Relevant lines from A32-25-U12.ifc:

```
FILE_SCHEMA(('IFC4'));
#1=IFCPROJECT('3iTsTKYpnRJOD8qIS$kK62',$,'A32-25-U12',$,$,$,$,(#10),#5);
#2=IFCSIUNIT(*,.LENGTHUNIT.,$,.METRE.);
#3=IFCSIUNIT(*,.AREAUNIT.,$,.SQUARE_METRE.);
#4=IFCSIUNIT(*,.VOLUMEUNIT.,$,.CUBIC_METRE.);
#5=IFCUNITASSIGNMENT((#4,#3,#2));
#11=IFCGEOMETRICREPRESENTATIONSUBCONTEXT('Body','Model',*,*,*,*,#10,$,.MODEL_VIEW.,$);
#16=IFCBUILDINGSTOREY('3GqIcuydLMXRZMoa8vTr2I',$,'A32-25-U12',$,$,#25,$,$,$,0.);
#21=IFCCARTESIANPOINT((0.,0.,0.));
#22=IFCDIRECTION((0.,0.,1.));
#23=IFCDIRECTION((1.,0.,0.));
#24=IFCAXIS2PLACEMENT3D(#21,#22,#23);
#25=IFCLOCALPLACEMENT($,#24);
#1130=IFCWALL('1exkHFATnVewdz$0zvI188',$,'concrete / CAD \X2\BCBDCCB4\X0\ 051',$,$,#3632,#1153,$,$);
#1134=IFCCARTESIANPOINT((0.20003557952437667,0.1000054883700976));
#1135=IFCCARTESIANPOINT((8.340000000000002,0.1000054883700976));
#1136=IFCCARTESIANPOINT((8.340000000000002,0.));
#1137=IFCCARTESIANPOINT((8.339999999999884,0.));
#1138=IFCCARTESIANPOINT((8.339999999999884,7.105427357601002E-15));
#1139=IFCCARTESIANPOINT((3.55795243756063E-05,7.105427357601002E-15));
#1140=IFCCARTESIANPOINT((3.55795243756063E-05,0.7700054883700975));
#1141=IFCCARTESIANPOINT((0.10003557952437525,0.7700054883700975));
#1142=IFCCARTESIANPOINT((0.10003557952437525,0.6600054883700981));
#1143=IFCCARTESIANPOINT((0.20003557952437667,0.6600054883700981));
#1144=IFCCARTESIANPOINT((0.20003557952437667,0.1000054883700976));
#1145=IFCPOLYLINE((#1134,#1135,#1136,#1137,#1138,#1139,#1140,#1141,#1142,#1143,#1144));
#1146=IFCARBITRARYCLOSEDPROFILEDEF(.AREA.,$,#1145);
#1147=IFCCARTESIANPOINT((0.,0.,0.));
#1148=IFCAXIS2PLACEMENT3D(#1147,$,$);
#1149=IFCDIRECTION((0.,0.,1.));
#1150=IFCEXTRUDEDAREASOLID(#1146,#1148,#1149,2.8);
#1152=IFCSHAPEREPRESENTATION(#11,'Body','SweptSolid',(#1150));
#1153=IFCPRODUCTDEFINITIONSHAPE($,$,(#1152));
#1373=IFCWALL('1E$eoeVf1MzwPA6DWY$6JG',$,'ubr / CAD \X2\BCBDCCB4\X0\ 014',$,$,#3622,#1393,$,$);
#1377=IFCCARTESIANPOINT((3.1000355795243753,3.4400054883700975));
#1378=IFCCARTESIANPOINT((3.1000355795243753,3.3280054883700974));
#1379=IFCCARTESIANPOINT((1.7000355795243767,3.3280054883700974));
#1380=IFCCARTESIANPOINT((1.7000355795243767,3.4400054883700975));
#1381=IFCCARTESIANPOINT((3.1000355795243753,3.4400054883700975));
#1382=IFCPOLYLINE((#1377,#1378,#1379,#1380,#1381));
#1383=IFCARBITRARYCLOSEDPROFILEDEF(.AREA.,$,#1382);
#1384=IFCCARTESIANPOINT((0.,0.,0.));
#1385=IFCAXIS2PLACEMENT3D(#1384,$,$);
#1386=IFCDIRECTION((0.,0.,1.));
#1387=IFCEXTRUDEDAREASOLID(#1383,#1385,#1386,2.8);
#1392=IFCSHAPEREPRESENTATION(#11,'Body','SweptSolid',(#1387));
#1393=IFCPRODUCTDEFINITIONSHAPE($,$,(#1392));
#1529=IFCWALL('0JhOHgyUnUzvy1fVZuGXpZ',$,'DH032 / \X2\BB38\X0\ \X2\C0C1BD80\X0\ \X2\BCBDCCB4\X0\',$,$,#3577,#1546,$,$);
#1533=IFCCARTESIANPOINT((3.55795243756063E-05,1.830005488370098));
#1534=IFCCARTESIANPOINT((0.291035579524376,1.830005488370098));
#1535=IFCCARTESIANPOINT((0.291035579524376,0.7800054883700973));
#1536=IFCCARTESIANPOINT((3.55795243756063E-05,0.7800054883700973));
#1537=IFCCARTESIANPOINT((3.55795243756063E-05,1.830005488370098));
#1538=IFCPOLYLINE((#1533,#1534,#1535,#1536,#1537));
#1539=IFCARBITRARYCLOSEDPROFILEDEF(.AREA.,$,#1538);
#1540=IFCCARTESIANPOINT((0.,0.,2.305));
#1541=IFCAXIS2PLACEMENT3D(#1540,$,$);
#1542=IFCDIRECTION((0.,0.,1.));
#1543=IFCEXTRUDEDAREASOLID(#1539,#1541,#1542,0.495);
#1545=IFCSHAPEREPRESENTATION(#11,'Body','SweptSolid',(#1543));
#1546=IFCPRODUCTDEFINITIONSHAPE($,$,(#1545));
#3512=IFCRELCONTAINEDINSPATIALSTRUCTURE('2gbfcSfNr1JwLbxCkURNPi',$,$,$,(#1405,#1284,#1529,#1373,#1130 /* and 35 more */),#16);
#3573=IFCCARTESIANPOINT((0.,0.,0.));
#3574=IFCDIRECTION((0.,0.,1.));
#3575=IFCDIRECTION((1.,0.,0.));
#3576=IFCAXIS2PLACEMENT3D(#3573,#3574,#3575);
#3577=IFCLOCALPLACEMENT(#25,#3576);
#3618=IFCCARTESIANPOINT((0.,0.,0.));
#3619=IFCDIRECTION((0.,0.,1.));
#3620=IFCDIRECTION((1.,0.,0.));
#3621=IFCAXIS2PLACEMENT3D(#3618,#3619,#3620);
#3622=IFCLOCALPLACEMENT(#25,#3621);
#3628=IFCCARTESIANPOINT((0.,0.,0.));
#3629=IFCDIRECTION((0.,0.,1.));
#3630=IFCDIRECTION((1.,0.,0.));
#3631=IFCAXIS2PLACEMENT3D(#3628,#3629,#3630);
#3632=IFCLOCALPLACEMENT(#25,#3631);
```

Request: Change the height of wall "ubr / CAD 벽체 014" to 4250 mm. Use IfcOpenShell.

```python
import ifcopenshell
import ifcopenshell.geom
import ifcopenshell.util.representation
import ifcopenshell.util.shape
import ifcopenshell.util.unit

model = ifcopenshell.open("A32-25-U12.ifc")
unit_scale = ifcopenshell.util.unit.calculate_unit_scale(model)
settings = ifcopenshell.geom.settings()


def volume(element):
    """Net volume in cubic metres, openings subtracted."""
    shape = ifcopenshell.geom.create_shape(settings, element)
    return ifcopenshell.util.shape.get_volume(shape.geometry)


wall = model.by_guid("1E$eoeVf1MzwPA6DWY$6JG")
before = volume(wall)

body = ifcopenshell.util.representation.get_representation(wall, "Model", "Body")
solid = body.Items[0]
old_height = solid.Depth
solid.Depth = 4.25 / unit_scale
after = volume(wall)

print(f"height {old_height:g} -> {solid.Depth:g}, volume {before:.3f} -> {after:.3f} m3")

model.write("A32-25-U12_rev.ifc")
```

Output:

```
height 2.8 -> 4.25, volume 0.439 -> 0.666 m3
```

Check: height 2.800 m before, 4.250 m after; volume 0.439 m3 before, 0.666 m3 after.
